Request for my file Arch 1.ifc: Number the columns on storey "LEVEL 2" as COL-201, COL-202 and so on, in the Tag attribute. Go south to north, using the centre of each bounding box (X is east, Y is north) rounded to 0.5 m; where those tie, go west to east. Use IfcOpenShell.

First a look at what the model holds.

```python
import ifcopenshell
import ifcopenshell.util.element
import ifcopenshell.util.placement

model = ifcopenshell.open("my file Arch 1.ifc")
print(model.schema)
storey = next(s for s in model.by_type("IfcBuildingStorey") if s.Name == "LEVEL 2")
columns = [e for e in ifcopenshell.util.element.get_decomposition(storey) if e.is_a("IfcColumn")]
for e in sorted(columns, key=lambda e: e.id()):
    origin = ifcopenshell.util.placement.get_local_placement(e.ObjectPlacement)[:3, 3]
    print(e.id(), e.Tag, e.Name, origin.round(2) + 0.0, sep=" | ")
```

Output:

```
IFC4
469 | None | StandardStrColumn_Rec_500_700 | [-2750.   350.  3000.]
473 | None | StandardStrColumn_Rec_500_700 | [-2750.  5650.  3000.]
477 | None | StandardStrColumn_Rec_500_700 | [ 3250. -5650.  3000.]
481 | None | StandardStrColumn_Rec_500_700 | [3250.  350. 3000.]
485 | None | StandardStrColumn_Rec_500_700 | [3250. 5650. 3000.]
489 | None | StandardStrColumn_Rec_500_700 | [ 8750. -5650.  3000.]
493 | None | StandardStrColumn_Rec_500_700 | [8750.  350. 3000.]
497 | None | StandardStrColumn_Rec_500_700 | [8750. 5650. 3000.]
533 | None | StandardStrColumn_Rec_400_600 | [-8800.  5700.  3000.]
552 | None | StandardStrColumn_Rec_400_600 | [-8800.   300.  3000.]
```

```python
import ifcopenshell
import ifcopenshell.geom
import ifcopenshell.util.element
import ifcopenshell.util.shape

model = ifcopenshell.open("my file Arch 1.ifc")
settings = ifcopenshell.geom.settings()
settings.set("use-world-coords", True)


def centre(element):
    shape = ifcopenshell.geom.create_shape(settings, element)
    return ifcopenshell.util.shape.get_bbox_centroid(shape.geometry)


storey = next(s for s in model.by_type("IfcBuildingStorey") if s.Name == "LEVEL 2")
columns = [e for e in ifcopenshell.util.element.get_decomposition(storey) if e.is_a("IfcColumn")]

# Insertion points can sit at a corner or the storey origin, so sort by the geometry (in metres).
centres = {e: centre(e) for e in columns}
columns.sort(key=lambda e: (round(centres[e][1] / 0.5), centres[e][0]))

for i, e in enumerate(columns, start=1):
    number = f"COL-2{i:02d}"
    e.Tag = number
    print(e.id(), number)

model.write("my file Arch 1_v2.ifc")
```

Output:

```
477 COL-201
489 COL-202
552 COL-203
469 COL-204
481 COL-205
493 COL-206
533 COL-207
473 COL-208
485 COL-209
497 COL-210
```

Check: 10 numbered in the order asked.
